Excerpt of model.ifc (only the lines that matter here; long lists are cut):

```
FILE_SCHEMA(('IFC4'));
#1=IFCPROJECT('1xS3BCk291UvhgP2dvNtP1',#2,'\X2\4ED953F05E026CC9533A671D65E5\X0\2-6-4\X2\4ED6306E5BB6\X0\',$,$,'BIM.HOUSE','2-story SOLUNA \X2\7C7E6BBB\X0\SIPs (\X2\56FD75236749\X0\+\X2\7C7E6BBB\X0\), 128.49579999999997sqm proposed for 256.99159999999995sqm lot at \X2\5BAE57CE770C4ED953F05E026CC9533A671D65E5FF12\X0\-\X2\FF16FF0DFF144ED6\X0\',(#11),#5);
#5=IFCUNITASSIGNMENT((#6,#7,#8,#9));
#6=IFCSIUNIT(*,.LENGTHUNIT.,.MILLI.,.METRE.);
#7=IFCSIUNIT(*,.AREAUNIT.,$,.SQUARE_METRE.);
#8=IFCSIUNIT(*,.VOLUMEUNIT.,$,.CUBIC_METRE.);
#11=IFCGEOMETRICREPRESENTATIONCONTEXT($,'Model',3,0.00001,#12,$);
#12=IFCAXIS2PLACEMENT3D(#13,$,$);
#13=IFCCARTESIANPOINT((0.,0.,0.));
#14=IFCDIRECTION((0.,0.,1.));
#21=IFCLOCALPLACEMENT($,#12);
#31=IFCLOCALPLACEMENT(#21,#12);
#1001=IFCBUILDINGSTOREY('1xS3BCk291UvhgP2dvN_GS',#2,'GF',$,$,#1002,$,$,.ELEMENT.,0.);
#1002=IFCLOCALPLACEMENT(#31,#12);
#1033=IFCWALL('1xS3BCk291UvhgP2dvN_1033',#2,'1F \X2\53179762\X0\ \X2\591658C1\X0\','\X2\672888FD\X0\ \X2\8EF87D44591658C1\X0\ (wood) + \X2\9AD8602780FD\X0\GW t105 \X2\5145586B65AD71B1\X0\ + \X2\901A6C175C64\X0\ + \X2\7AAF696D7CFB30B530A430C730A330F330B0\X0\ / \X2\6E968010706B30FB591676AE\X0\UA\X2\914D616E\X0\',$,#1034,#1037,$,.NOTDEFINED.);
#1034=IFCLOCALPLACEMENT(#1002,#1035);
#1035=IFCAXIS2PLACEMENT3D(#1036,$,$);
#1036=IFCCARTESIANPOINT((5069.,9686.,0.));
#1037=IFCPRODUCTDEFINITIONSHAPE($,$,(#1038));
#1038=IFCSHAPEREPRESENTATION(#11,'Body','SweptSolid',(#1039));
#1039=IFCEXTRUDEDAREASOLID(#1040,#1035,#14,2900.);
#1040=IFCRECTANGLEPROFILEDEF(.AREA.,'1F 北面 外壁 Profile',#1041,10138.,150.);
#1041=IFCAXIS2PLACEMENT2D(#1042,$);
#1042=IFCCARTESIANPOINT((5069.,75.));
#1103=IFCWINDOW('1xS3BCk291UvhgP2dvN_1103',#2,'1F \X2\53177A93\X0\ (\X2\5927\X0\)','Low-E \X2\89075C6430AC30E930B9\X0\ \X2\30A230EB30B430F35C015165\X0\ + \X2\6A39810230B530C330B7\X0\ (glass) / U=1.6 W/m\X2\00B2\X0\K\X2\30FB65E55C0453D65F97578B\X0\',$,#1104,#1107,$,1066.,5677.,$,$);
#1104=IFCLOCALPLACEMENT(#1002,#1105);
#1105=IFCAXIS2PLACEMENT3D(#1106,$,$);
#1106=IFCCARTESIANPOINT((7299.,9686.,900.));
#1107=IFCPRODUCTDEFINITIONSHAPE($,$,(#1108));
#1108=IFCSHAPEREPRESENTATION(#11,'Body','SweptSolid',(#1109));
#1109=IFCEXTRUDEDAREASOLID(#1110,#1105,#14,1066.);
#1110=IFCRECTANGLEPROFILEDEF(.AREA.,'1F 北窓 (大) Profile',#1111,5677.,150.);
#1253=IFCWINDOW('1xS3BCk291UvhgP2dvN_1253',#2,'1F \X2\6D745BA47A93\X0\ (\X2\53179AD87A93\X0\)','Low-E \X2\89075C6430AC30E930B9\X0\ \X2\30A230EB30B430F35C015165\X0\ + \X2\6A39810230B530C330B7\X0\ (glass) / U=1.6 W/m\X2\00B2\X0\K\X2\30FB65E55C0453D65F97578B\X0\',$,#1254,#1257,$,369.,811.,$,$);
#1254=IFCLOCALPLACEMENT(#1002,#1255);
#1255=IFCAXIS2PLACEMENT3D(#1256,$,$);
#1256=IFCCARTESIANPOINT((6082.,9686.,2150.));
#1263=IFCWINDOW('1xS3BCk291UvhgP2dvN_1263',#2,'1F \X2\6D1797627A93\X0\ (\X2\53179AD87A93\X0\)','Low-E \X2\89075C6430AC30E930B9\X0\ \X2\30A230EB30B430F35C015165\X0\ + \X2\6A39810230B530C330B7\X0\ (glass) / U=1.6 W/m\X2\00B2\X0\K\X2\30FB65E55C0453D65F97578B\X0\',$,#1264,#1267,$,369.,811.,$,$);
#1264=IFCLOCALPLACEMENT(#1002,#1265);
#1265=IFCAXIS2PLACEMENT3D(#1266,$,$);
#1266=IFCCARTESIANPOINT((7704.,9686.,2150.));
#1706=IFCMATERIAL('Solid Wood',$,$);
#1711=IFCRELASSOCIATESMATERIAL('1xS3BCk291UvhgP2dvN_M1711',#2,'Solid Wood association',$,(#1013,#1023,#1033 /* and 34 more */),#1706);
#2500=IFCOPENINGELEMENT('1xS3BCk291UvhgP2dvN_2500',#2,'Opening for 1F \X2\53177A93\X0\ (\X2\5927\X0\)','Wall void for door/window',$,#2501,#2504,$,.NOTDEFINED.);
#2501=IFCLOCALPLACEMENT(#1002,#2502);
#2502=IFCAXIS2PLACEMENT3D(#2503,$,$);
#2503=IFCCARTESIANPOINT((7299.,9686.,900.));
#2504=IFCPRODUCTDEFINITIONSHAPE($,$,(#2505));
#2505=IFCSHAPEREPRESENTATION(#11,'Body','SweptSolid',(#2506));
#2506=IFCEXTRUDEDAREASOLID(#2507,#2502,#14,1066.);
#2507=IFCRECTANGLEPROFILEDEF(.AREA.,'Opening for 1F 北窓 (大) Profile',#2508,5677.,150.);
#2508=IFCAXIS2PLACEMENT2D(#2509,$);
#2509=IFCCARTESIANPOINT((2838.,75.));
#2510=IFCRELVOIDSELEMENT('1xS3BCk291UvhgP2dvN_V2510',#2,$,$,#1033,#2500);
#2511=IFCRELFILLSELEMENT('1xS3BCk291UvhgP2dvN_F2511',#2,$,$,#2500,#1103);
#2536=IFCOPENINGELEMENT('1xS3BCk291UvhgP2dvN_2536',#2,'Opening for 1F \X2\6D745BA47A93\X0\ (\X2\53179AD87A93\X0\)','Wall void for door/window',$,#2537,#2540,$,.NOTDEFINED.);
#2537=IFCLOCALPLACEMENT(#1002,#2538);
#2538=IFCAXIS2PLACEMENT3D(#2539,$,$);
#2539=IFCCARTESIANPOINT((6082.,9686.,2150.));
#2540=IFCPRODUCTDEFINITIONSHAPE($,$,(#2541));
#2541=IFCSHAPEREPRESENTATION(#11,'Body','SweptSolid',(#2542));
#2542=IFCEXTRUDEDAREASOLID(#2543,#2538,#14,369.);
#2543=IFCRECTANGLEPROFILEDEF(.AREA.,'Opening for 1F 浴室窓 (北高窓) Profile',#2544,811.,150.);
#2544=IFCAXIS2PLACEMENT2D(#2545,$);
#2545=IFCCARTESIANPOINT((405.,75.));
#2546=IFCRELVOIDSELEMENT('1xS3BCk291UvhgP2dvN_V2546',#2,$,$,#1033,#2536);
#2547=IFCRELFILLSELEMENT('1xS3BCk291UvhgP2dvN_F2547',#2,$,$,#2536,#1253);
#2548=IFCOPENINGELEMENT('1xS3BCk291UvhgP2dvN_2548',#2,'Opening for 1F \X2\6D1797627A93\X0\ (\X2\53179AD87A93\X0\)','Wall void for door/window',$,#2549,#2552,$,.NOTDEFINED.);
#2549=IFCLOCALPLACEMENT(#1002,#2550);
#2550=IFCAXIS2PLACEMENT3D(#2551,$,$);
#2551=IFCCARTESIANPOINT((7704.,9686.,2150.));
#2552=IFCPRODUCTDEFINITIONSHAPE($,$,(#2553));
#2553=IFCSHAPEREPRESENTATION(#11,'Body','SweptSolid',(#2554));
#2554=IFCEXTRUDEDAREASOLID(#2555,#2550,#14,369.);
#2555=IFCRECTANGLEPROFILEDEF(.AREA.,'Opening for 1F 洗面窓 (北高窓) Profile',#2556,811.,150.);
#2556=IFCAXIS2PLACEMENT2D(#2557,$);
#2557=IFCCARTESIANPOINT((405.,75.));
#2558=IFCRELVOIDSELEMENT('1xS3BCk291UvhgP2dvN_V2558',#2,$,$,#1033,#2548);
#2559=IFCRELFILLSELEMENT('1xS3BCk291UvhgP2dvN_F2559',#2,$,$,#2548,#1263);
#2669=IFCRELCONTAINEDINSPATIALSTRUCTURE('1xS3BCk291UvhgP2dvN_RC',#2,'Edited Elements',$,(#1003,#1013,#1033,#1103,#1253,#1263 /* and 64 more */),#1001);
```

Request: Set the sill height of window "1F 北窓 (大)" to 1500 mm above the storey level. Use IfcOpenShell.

```python
import numpy as np
import ifcopenshell
import ifcopenshell.api.geometry
import ifcopenshell.geom
import ifcopenshell.util.element
import ifcopenshell.util.placement
import ifcopenshell.util.shape
import ifcopenshell.util.unit

model = ifcopenshell.open("model.ifc")
unit_scale = ifcopenshell.util.unit.calculate_unit_scale(model)

window = model.by_guid("1xS3BCk291UvhgP2dvN_1103")
opening = window.FillsVoids[0].RelatingOpeningElement
storey = ifcopenshell.util.element.get_container(window, ifc_class="IfcBuildingStorey")
level = ifcopenshell.util.placement.get_local_placement(storey.ObjectPlacement)[2, 3]

# The opening's origin need not be at the sill, so measure its lowest point.
shape = ifcopenshell.geom.create_shape(ifcopenshell.geom.settings(), opening)
bottom = ifcopenshell.util.shape.get_shape_bottom_elevation(shape, shape.geometry) / unit_scale
dz = level + 1500.0 - bottom

shift = np.array([0.0, 0.0, dz])
# The window is not placed relative to its opening, so move both.
for product in (opening, window):
    matrix = ifcopenshell.util.placement.get_local_placement(product.ObjectPlacement)
    matrix[:3, 3] += shift
    ifcopenshell.api.geometry.edit_object_placement(model, product=product, matrix=matrix, is_si=False)

print(f"moved by {dz * unit_scale:+.3f} m")

model.write("model_v2.ifc")
```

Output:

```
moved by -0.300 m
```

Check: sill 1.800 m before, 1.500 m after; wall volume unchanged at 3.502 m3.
